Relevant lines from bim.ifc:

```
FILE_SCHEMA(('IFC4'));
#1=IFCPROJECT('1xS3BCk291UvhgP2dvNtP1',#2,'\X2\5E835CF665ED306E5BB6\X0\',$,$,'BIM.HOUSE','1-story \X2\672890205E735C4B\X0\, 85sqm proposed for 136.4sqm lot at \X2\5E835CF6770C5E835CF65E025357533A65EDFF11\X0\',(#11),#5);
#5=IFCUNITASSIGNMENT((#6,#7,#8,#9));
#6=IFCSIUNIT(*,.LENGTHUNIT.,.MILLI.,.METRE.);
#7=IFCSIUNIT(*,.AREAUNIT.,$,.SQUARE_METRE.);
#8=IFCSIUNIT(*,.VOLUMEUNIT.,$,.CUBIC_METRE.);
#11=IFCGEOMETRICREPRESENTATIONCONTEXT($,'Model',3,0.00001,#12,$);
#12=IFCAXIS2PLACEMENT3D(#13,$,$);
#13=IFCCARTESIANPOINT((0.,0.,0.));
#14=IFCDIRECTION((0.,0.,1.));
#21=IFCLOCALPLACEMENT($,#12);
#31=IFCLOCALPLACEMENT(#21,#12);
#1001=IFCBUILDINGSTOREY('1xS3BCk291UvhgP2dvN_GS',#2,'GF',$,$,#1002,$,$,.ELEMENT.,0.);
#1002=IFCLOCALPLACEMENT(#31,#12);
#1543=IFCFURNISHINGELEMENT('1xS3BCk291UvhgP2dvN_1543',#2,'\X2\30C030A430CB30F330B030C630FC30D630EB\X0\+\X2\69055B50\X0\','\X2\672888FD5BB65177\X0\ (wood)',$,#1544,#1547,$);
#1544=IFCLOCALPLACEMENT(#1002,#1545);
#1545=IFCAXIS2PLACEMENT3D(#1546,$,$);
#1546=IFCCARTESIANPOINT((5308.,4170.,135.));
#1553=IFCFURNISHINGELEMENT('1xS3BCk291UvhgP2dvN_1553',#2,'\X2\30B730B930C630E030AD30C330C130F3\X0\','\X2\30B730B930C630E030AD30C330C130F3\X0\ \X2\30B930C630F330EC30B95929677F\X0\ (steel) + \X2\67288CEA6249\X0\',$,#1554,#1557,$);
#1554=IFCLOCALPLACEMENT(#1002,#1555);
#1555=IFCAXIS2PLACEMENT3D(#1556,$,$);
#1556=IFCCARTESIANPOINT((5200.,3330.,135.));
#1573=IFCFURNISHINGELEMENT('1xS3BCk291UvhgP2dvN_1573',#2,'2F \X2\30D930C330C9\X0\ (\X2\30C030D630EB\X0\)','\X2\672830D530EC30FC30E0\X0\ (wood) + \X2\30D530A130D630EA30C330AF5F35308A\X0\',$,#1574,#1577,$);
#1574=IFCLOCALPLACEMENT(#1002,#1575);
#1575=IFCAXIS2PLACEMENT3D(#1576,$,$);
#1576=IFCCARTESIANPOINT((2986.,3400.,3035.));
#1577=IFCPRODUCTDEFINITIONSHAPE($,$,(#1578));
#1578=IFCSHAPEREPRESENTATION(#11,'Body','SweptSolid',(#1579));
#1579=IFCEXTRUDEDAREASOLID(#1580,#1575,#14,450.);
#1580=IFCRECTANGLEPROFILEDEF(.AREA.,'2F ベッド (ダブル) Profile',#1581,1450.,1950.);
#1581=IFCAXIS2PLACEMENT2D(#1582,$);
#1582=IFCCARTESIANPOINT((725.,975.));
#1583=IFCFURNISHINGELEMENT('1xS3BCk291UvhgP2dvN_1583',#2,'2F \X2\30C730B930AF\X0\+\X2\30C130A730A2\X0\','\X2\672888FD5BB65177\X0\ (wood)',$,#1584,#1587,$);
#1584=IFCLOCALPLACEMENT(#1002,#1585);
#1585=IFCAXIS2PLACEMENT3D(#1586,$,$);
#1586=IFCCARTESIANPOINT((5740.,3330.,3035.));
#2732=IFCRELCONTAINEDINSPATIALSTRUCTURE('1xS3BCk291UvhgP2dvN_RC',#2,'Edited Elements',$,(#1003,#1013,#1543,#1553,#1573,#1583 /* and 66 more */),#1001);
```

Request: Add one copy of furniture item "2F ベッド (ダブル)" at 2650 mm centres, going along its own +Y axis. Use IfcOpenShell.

```python
import ifcopenshell
import ifcopenshell.api.geometry
import ifcopenshell.api.root
import ifcopenshell.util.element
import ifcopenshell.util.placement
import ifcopenshell.util.unit

model = ifcopenshell.open("bim.ifc")
unit_scale = ifcopenshell.util.unit.calculate_unit_scale(model)


def reuse_history(source, copy):
    """copy_class also copies each property set's owner history, people and application; keep the originals."""
    for rel in copy.IsDefinedBy:
        if rel.is_a("IfcRelDefinesByProperties") and (history := rel.RelatingPropertyDefinition.OwnerHistory):
            rel.RelatingPropertyDefinition.OwnerHistory = source.OwnerHistory
            ifcopenshell.util.element.remove_deep2(model, history)


source = model.by_guid("1xS3BCk291UvhgP2dvN_1573")
base = ifcopenshell.util.placement.get_local_placement(source.ObjectPlacement)
step = base[:3, 1] * 2.65 / unit_scale

for i in range(1, 2):
    copy = ifcopenshell.api.root.copy_class(model, product=source)
    copy.Representation = ifcopenshell.util.element.copy_deep(
        model, source.Representation, exclude=["IfcGeometricRepresentationContext", "IfcRepresentationMap"]
    )
    reuse_history(source, copy)
    matrix = base.copy()
    matrix[:3, 3] += i * step
    print("added at", matrix[:3, 3].round(3) + 0.0)
    ifcopenshell.api.geometry.edit_object_placement(model, product=copy, matrix=matrix, is_si=False)

model.write("bim_rev.ifc")
```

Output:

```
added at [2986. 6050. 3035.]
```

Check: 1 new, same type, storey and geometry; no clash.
